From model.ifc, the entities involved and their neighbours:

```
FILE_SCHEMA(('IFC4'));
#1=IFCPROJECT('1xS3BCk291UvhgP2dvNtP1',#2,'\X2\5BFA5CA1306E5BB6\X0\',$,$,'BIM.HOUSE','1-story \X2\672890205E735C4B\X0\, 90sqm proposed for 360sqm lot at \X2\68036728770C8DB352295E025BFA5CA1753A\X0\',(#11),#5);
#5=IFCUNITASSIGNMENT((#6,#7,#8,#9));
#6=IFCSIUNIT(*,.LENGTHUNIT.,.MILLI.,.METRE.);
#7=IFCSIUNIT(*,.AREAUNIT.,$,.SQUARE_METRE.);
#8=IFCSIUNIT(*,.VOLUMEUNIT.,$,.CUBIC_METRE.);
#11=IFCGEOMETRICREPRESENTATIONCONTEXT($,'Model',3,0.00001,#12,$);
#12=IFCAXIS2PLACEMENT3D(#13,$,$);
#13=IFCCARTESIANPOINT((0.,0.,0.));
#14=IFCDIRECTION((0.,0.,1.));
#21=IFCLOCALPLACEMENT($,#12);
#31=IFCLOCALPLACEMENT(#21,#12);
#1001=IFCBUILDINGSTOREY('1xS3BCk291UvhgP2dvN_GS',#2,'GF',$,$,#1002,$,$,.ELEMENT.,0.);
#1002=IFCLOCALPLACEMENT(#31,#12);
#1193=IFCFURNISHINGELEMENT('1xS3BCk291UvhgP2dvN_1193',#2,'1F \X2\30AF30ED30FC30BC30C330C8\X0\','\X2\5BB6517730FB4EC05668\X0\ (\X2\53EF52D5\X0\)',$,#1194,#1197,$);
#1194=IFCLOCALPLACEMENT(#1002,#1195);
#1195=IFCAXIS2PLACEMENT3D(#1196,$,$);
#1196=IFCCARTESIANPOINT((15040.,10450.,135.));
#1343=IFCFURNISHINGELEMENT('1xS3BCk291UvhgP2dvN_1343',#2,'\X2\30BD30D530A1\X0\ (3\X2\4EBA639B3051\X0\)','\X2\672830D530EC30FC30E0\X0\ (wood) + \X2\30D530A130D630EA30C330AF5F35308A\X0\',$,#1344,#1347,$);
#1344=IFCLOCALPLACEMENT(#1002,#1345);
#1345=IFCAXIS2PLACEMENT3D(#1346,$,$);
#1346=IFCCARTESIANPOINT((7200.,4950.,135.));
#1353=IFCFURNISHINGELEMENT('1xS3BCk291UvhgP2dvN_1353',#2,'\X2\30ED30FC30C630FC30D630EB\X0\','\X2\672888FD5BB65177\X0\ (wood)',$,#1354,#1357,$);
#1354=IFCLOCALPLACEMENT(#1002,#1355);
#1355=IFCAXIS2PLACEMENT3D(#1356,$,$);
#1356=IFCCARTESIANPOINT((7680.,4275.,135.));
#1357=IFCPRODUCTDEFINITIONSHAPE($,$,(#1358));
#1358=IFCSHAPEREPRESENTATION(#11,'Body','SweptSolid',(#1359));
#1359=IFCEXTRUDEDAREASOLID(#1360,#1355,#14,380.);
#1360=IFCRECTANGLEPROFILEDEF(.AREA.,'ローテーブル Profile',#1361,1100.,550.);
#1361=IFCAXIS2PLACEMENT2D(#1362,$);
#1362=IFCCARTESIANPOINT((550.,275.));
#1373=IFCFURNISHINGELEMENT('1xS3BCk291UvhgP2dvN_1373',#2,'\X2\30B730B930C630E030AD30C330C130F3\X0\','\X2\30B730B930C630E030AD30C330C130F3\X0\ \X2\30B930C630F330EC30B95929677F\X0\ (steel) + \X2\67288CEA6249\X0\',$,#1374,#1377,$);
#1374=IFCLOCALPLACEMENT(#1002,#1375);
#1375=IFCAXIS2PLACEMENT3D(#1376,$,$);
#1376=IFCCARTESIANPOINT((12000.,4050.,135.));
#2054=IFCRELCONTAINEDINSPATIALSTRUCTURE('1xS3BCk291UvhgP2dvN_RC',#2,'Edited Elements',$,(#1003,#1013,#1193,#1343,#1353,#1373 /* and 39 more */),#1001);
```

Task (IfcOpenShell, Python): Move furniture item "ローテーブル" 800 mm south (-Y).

```python
import ifcopenshell
import ifcopenshell.api.geometry
import ifcopenshell.util.placement

model = ifcopenshell.open("model.ifc")

item = model.by_id(1353)
matrix = ifcopenshell.util.placement.get_local_placement(item.ObjectPlacement)
matrix[1, 3] -= 800.0
ifcopenshell.api.geometry.edit_object_placement(model, product=item, matrix=matrix, is_si=False)

print(ifcopenshell.util.placement.get_local_placement(item.ObjectPlacement).round(3) + 0.0)

model.write("model_rev.ifc")
```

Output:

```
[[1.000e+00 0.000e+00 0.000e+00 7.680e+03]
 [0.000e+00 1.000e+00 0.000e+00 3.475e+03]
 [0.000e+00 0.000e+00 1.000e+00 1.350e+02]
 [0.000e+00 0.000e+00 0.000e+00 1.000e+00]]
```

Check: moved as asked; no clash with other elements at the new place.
